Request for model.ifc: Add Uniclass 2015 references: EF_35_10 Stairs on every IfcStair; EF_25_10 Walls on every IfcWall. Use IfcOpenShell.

First a look at what the model holds.

```python
import ifcopenshell

model = ifcopenshell.open("model.ifc")
print(model.schema)
print("classifications:", [c.Name for c in model.by_type("IfcClassification")])
for ifc_class in ("IfcDoor", "IfcRoof", "IfcStair", "IfcWall", "IfcWindow"):
    print(ifc_class, len(model.by_type(ifc_class)))
```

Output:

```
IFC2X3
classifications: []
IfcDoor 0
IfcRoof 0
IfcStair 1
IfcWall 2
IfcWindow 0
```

```python
import ifcopenshell
import ifcopenshell.api.classification

model = ifcopenshell.open("model.ifc")

# IFC2X3 requires Source and Edition and has no link from the project to the system.
system = model.create_entity("IfcClassification", Source="NBS", Edition="2015", Name="Uniclass 2015")

codes = {
    "IfcStair": ("EF_35_10", "Stairs"),
    "IfcWall": ("EF_25_10", "Walls"),
}
for ifc_class, (code, name) in codes.items():
    products = model.by_type(ifc_class)
    ifcopenshell.api.classification.add_reference(
        model, products=products, classification=system, identification=code, name=name
    )
    print(code, len(products))

model.write("model_v2.ifc")
```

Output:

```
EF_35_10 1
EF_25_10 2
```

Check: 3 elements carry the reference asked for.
